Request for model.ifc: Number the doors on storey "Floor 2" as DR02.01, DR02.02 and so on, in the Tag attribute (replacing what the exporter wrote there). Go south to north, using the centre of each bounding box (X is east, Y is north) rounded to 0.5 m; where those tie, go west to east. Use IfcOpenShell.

First a look at what the model holds.

```python
import ifcopenshell
import ifcopenshell.util.element
import ifcopenshell.util.placement

model = ifcopenshell.open("model.ifc")
print(model.schema)
storey = next(s for s in model.by_type("IfcBuildingStorey") if s.Name == "Floor 2")
doors = [e for e in ifcopenshell.util.element.get_decomposition(storey) if e.is_a("IfcDoor")]
for e in sorted(doors, key=lambda e: e.id()):
    origin = ifcopenshell.util.placement.get_local_placement(e.ObjectPlacement)[:3, 3]
    print(e.id(), e.Tag, e.Name, origin.round(2) + 0.0, sep=" | ")
```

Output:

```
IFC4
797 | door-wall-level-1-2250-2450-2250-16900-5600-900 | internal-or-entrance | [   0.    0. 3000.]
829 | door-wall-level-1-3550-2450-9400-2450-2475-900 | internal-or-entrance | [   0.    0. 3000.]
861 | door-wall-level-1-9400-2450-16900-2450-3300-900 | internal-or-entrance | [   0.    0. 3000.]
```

```python
import ifcopenshell
import ifcopenshell.geom
import ifcopenshell.util.element
import ifcopenshell.util.shape

model = ifcopenshell.open("model.ifc")
settings = ifcopenshell.geom.settings()
settings.set("use-world-coords", True)


def centre(element):
    shape = ifcopenshell.geom.create_shape(settings, element)
    return ifcopenshell.util.shape.get_bbox_centroid(shape.geometry)


storey = next(s for s in model.by_type("IfcBuildingStorey") if s.Name == "Floor 2")
doors = [e for e in ifcopenshell.util.element.get_decomposition(storey) if e.is_a("IfcDoor")]

# Insertion points can sit at a corner or the storey origin, so sort by the geometry (in metres).
centres = {e: centre(e) for e in doors}
doors.sort(key=lambda e: (round(centres[e][1] / 0.5), centres[e][0]))

for i, e in enumerate(doors, start=1):
    number = f"DR02.{i:02d}"
    e.Tag = number
    print(e.id(), number)

model.write("model-out.ifc")
```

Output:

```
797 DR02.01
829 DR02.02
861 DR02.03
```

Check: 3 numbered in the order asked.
